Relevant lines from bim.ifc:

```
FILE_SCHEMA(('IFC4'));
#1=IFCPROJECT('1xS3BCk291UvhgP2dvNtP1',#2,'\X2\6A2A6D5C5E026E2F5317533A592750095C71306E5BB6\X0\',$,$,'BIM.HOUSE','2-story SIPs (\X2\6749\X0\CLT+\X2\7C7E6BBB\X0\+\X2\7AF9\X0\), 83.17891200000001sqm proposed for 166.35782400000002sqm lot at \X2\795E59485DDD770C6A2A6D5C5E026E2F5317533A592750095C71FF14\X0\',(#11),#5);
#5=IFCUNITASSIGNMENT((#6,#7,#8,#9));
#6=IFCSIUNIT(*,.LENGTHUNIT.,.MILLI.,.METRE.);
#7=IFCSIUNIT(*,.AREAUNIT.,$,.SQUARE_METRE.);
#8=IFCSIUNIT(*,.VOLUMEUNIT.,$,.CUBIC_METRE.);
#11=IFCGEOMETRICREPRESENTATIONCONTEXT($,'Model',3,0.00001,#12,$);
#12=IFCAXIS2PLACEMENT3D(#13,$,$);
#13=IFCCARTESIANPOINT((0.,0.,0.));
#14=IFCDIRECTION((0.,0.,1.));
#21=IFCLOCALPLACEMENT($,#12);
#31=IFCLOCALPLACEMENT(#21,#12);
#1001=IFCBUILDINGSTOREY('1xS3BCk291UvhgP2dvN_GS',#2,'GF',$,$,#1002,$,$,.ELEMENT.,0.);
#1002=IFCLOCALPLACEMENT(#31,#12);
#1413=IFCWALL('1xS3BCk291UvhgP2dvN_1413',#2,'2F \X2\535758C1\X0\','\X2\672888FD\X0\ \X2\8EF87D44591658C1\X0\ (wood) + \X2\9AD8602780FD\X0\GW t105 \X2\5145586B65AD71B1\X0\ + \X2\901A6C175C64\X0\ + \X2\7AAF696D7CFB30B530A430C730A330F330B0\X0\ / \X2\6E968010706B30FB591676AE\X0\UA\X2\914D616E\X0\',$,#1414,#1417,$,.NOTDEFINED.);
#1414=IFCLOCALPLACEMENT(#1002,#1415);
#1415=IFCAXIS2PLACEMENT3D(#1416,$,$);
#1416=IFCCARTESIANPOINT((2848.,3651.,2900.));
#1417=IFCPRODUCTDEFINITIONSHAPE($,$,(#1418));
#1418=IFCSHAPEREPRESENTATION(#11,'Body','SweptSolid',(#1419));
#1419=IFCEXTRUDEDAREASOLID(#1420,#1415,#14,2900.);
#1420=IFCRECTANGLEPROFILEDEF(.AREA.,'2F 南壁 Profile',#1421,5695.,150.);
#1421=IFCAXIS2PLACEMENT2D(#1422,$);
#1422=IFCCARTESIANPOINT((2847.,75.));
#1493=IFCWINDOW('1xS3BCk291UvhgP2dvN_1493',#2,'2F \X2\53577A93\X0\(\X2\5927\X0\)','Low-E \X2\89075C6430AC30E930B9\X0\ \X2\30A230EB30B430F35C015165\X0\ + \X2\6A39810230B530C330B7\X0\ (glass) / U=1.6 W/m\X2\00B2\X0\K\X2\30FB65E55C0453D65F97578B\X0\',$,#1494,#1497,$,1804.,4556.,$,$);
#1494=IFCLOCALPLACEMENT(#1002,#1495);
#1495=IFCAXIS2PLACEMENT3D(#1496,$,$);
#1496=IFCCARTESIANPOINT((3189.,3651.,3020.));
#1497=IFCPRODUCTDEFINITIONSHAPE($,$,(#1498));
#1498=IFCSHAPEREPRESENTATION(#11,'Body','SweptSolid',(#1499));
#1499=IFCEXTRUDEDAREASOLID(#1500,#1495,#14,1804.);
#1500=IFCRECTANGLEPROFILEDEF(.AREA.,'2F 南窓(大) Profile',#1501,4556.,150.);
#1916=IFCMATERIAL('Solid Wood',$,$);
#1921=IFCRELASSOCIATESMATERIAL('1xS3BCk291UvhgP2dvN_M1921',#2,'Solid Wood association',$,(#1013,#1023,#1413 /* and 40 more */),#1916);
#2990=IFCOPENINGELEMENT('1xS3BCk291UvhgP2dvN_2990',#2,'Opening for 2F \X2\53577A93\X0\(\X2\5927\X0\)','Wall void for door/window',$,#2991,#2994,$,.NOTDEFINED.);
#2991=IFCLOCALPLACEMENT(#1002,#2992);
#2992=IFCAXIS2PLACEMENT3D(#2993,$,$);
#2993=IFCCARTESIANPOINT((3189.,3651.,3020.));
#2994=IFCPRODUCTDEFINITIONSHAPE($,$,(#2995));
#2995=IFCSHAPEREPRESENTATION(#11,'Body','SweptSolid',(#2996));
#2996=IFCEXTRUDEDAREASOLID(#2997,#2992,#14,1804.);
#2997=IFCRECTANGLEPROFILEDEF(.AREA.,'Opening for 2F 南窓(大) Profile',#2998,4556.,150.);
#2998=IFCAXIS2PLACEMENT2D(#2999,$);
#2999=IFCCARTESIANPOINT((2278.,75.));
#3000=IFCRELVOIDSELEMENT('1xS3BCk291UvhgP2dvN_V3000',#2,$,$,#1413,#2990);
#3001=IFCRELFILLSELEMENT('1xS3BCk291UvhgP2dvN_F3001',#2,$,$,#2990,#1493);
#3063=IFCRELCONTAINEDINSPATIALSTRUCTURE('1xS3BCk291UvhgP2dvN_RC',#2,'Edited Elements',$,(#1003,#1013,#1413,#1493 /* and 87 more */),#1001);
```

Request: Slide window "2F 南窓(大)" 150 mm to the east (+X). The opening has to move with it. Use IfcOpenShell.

```python
import ifcopenshell
import ifcopenshell.api.geometry
import ifcopenshell.util.placement
import ifcopenshell.util.unit

model = ifcopenshell.open("bim.ifc")
unit_scale = ifcopenshell.util.unit.calculate_unit_scale(model)

window = model.by_id(1493)
opening = window.FillsVoids[0].RelatingOpeningElement
wall = opening.VoidsElements[0].RelatingBuildingElement

wall_matrix = ifcopenshell.util.placement.get_local_placement(wall.ObjectPlacement)
shift = wall_matrix[:3, 0] * 0.15 / unit_scale
before = ifcopenshell.util.placement.get_local_placement(window.ObjectPlacement)[:3, 3].copy()

# The window is not placed relative to its opening, so move both.
for product in (opening, window):
    matrix = ifcopenshell.util.placement.get_local_placement(product.ObjectPlacement)
    matrix[:3, 3] += shift
    ifcopenshell.api.geometry.edit_object_placement(model, product=product, matrix=matrix, is_si=False)

after = ifcopenshell.util.placement.get_local_placement(window.ObjectPlacement)[:3, 3]
print("window moved by", (after - before).round(3) + 0.0)

model.write("bim-out.ifc")
```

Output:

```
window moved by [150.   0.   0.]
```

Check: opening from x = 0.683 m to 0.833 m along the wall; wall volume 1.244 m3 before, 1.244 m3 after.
